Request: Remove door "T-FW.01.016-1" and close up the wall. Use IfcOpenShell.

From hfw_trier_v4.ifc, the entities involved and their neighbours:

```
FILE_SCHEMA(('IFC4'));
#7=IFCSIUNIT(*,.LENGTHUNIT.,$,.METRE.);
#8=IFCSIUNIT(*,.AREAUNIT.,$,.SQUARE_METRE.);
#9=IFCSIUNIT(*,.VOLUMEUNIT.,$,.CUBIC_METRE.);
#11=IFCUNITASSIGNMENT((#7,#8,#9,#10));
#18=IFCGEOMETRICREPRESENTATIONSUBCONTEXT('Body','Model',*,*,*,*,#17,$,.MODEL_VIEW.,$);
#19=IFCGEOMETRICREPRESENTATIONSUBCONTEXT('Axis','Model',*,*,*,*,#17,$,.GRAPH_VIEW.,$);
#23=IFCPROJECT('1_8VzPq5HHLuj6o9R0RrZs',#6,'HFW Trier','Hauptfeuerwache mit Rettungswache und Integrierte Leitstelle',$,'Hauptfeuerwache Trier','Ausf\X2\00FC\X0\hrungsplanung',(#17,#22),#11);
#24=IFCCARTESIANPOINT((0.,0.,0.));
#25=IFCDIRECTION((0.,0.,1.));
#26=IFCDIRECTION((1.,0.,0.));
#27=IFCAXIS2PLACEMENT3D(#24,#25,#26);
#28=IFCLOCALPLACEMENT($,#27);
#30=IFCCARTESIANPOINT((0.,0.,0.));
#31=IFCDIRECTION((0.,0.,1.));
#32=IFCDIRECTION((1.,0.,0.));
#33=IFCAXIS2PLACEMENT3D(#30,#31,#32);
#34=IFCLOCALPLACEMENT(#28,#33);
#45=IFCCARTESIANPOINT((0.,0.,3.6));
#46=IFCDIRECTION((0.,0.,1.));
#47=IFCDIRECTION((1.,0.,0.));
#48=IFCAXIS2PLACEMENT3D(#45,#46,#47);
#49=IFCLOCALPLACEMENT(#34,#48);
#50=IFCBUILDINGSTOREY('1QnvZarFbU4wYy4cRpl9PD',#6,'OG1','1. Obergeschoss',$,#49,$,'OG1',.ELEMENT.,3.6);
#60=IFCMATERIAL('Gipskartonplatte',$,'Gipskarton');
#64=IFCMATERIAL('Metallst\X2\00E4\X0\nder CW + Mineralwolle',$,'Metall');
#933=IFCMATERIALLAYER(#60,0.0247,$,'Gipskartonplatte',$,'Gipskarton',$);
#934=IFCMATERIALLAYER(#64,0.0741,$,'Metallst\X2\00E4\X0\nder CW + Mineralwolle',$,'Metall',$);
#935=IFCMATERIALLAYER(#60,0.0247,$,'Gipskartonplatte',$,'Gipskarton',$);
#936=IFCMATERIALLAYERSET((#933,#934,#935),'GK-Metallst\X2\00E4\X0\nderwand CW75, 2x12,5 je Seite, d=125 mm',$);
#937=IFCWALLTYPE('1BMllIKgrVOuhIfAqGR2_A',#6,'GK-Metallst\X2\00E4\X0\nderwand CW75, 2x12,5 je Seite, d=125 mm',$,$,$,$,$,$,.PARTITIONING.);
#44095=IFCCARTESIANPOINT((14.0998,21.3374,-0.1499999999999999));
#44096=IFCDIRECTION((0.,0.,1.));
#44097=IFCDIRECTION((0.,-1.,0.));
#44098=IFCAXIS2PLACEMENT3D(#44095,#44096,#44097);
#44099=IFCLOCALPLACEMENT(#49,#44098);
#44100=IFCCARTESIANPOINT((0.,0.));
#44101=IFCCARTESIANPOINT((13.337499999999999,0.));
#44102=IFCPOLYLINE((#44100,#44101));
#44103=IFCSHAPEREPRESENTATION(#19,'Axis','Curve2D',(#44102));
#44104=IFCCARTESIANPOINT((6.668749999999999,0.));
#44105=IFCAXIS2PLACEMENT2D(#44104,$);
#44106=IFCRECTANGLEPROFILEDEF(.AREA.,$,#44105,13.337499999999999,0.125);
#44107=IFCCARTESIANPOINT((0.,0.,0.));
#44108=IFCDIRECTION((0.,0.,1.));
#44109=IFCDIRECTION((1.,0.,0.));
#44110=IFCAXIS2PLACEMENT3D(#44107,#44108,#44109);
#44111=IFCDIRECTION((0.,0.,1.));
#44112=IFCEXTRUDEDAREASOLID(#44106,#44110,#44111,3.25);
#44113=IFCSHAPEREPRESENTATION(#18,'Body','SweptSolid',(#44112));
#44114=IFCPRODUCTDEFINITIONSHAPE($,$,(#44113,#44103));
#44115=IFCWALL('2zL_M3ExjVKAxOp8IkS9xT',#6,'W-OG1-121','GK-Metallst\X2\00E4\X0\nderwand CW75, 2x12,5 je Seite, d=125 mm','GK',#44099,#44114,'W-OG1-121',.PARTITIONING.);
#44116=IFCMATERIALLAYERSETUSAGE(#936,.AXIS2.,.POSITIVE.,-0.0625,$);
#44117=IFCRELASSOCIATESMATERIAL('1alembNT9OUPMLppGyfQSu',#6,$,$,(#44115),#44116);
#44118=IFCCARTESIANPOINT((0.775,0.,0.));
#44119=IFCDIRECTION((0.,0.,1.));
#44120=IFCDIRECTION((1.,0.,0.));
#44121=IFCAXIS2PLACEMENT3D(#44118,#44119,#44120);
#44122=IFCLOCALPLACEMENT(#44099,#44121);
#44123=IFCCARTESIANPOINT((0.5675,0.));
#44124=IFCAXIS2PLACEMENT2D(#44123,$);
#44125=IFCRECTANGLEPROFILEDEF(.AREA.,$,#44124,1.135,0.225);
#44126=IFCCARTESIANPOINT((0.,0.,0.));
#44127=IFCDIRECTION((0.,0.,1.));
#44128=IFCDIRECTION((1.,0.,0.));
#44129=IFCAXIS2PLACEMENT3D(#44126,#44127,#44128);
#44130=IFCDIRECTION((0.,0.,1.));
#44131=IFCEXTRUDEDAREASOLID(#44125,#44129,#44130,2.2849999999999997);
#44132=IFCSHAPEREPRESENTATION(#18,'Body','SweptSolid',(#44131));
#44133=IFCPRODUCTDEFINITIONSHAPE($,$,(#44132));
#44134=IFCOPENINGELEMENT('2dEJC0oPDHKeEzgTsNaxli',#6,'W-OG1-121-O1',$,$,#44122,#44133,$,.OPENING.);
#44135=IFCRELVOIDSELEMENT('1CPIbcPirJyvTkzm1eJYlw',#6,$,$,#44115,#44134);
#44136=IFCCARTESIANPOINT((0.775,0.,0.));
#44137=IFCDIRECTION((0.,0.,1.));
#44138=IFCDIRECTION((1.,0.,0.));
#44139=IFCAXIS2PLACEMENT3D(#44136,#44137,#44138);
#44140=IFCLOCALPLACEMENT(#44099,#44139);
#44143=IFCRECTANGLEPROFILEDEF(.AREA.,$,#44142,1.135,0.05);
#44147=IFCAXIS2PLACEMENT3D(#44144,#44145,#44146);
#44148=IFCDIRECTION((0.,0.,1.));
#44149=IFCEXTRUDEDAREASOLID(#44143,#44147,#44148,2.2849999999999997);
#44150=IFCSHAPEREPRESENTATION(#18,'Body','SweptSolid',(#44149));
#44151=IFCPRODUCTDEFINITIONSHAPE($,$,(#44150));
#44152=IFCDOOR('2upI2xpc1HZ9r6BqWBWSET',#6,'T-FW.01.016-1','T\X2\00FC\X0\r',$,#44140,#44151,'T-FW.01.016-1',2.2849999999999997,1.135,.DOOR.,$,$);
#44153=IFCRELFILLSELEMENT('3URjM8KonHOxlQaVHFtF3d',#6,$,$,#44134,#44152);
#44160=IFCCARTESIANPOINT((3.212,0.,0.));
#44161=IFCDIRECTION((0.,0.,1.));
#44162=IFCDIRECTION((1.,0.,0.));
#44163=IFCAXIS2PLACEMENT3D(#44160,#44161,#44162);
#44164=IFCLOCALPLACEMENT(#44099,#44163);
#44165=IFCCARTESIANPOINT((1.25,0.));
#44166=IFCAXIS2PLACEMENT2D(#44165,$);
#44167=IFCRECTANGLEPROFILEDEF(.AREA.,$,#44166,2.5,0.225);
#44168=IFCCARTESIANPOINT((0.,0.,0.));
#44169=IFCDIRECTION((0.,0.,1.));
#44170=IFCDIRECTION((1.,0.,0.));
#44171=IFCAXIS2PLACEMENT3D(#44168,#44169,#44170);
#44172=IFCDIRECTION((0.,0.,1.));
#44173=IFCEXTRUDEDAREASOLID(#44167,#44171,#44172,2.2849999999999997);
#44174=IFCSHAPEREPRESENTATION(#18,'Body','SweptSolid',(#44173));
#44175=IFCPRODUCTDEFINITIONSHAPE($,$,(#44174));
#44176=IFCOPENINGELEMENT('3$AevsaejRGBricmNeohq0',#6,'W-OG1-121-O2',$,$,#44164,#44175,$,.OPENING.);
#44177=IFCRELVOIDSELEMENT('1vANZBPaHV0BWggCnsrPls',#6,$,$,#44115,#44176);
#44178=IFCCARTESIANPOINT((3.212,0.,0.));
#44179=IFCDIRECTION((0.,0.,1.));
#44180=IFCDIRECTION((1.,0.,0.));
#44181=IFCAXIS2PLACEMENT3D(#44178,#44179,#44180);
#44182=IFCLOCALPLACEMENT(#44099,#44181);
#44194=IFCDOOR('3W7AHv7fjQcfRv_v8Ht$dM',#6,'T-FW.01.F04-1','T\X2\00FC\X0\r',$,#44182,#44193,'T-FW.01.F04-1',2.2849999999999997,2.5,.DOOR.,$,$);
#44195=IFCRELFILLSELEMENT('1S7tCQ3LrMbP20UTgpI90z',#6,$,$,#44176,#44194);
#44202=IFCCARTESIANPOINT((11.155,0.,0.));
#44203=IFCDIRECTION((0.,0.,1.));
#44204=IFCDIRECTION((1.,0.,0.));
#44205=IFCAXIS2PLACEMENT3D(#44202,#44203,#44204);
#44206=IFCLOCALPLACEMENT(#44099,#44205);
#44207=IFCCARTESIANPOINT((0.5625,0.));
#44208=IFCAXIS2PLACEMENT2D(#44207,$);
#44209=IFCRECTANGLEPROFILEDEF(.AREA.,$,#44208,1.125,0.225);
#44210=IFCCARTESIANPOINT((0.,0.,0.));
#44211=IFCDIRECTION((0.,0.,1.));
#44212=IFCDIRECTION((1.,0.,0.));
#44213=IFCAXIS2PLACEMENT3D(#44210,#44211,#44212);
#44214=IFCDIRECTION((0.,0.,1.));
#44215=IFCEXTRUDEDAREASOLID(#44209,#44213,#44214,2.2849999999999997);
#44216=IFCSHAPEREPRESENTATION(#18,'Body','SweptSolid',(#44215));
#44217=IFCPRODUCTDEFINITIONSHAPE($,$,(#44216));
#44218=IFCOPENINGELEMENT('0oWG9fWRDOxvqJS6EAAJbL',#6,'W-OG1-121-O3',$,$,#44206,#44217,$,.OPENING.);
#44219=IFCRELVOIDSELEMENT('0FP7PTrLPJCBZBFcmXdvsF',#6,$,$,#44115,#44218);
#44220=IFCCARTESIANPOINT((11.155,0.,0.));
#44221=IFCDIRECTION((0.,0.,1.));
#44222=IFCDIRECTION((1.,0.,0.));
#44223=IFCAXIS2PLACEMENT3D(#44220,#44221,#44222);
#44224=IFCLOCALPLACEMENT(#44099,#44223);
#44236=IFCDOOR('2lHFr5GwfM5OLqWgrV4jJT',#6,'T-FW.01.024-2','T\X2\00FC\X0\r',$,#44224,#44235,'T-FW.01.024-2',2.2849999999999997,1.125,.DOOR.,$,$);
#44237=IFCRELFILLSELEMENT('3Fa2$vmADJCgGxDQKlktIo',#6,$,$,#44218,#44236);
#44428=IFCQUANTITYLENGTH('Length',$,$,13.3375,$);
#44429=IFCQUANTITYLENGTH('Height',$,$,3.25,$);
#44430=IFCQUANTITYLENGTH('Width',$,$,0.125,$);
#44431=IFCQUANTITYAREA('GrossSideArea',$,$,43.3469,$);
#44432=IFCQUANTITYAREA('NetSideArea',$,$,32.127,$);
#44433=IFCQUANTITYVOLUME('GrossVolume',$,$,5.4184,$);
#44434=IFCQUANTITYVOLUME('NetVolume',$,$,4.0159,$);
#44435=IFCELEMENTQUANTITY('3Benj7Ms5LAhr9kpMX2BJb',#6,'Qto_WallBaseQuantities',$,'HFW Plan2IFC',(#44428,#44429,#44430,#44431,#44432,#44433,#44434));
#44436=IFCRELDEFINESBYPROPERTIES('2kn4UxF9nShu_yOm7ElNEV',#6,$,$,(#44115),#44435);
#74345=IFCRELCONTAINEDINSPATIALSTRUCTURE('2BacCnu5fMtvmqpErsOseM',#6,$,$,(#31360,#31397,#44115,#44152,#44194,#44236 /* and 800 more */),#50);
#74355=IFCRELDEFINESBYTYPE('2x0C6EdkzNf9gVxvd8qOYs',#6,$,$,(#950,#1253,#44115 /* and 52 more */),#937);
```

```python
import ifcopenshell
import ifcopenshell.api.feature
import ifcopenshell.api.pset
import ifcopenshell.api.root
import ifcopenshell.geom
import ifcopenshell.util.element
import ifcopenshell.util.shape
import ifcopenshell.util.unit

model = ifcopenshell.open("hfw_trier_v4.ifc")
area_scale = ifcopenshell.util.unit.calculate_unit_scale(model, "AREAUNIT")
volume_scale = ifcopenshell.util.unit.calculate_unit_scale(model, "VOLUMEUNIT")
settings = ifcopenshell.geom.settings()


def volume(element):
    """Net volume in cubic metres, openings subtracted."""
    shape = ifcopenshell.geom.create_shape(settings, element)
    return ifcopenshell.util.shape.get_volume(shape.geometry)


door = model.by_guid("2upI2xpc1HZ9r6BqWBWSET")
opening = door.FillsVoids[0].RelatingOpeningElement
wall = opening.VoidsElements[0].RelatingBuildingElement
before = volume(wall)

ifcopenshell.api.root.remove_product(model, product=door)
ifcopenshell.api.feature.remove_feature(model, feature=opening)

after = volume(wall)
thickness = 0.125  # wall thickness in metres

# Update the wall's stored quantities.
qto = model.by_id(ifcopenshell.util.element.get_pset(wall, "Qto_WallBaseQuantities", should_inherit=False)["id"])
ifcopenshell.api.pset.edit_qto(model, qto=qto, properties={
    "NetSideArea": after / thickness / area_scale,
    "NetVolume": after / volume_scale,
})

print(f"wall volume {before:.3f} -> {after:.3f} m3")

model.write("hfw_trier_v4_v2.ifc")
```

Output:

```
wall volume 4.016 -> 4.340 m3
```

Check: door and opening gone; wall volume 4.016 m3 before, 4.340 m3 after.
